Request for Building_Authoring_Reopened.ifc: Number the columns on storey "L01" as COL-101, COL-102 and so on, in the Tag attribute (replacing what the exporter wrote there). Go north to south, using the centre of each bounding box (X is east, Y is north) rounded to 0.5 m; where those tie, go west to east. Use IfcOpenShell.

First a look at what the model holds.

```python
import ifcopenshell
import ifcopenshell.util.element
import ifcopenshell.util.placement

model = ifcopenshell.open("Building_Authoring_Reopened.ifc")
print(model.schema)
storey = next(s for s in model.by_type("IfcBuildingStorey") if s.Name == "L01")
columns = [e for e in ifcopenshell.util.element.get_decomposition(storey) if e.is_a("IfcColumn")]
for e in sorted(columns, key=lambda e: e.id()):
    origin = ifcopenshell.util.placement.get_local_placement(e.ObjectPlacement)[:3, 3]
    print(e.id(), e.Tag, e.Name, origin.round(2) + 0.0, sep=" | ")
```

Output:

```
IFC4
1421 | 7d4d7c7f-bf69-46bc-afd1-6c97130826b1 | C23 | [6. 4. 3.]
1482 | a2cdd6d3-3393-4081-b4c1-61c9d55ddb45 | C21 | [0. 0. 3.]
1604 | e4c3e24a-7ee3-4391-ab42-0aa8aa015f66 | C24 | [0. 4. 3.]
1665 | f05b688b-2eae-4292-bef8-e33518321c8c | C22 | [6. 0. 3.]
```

```python
import ifcopenshell
import ifcopenshell.geom
import ifcopenshell.util.element
import ifcopenshell.util.shape

model = ifcopenshell.open("Building_Authoring_Reopened.ifc")
settings = ifcopenshell.geom.settings()
settings.set("use-world-coords", True)


def centre(element):
    shape = ifcopenshell.geom.create_shape(settings, element)
    return ifcopenshell.util.shape.get_bbox_centroid(shape.geometry)


storey = next(s for s in model.by_type("IfcBuildingStorey") if s.Name == "L01")
columns = [e for e in ifcopenshell.util.element.get_decomposition(storey) if e.is_a("IfcColumn")]

# Insertion points can sit at a corner or the storey origin, so sort by the geometry (in metres).
centres = {e: centre(e) for e in columns}
columns.sort(key=lambda e: (-round(centres[e][1] / 0.5), centres[e][0]))

for i, e in enumerate(columns, start=1):
    number = f"COL-1{i:02d}"
    e.Tag = number
    print(e.id(), number)

model.write("Building_Authoring_Reopened_v2.ifc")
```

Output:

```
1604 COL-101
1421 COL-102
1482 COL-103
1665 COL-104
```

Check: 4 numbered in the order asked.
